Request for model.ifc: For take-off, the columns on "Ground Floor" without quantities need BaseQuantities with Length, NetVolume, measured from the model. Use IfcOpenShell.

First a look at what the model holds.

```python
import ifcopenshell
import ifcopenshell.util.element
import ifcopenshell.util.unit

model = ifcopenshell.open("model.ifc")
print(model.schema)
for unit_type in ("LENGTHUNIT", "AREAUNIT", "VOLUMEUNIT"):
    print(unit_type, ifcopenshell.util.unit.calculate_unit_scale(model, unit_type))
storey = next(s for s in model.by_type("IfcBuildingStorey") if s.Name == "Ground Floor")
columns = [e for e in ifcopenshell.util.element.get_decomposition(storey) if e.is_a("IfcColumn")]
for e in sorted(columns, key=lambda e: e.id()):
    print(e.id(), e.is_a(), e.Name, list(ifcopenshell.util.element.get_psets(e, qtos_only=True)), sep=" | ")
```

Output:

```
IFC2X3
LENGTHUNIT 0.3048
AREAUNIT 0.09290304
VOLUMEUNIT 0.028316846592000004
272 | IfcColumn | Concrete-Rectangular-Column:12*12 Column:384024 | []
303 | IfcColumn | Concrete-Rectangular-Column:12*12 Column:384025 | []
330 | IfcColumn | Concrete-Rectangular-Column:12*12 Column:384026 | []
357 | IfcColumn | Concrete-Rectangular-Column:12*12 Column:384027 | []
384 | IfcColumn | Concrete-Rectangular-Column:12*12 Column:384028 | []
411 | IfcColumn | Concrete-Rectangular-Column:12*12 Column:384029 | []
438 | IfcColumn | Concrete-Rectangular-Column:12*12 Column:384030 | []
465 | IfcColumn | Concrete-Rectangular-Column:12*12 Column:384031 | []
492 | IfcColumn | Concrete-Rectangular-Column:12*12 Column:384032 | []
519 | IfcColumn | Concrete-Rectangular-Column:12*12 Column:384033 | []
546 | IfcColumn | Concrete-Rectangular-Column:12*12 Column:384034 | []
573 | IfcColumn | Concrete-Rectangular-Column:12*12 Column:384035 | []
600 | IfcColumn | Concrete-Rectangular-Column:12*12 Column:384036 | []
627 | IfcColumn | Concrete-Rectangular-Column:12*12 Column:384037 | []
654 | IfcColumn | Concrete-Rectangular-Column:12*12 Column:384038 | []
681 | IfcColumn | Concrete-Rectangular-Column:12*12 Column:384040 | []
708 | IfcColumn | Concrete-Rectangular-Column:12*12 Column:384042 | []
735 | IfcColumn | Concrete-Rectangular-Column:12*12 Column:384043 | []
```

```python
import ifcopenshell
import ifcopenshell.api.pset
import ifcopenshell.geom
import ifcopenshell.util.element
import ifcopenshell.util.shape
import ifcopenshell.util.unit

model = ifcopenshell.open("model.ifc")
unit_scale = ifcopenshell.util.unit.calculate_unit_scale(model)
volume_scale = ifcopenshell.util.unit.calculate_unit_scale(model, "VOLUMEUNIT")
settings = ifcopenshell.geom.settings()

storey = next(s for s in model.by_type("IfcBuildingStorey") if s.Name == "Ground Floor")
columns = [e for e in ifcopenshell.util.element.get_decomposition(storey) if e.is_a("IfcColumn")]

for e in sorted(columns, key=lambda e: e.id()):
    if ifcopenshell.util.element.get_psets(e, qtos_only=True, should_inherit=False):
        continue
    # Geometry comes back in metres, in the element's own axes.
    shape = ifcopenshell.geom.create_shape(settings, e)
    values = {
        "Length": ifcopenshell.util.shape.get_z(shape.geometry) / unit_scale,
        "NetVolume": ifcopenshell.util.shape.get_volume(shape.geometry) / volume_scale,
    }
    qto = ifcopenshell.api.pset.add_qto(model, product=e, name="BaseQuantities")
    ifcopenshell.api.pset.edit_qto(model, qto=qto, properties=values)
    print(e.id(), {k: round(v, 3) for k, v in values.items()})

model.write("model_rev.ifc")
```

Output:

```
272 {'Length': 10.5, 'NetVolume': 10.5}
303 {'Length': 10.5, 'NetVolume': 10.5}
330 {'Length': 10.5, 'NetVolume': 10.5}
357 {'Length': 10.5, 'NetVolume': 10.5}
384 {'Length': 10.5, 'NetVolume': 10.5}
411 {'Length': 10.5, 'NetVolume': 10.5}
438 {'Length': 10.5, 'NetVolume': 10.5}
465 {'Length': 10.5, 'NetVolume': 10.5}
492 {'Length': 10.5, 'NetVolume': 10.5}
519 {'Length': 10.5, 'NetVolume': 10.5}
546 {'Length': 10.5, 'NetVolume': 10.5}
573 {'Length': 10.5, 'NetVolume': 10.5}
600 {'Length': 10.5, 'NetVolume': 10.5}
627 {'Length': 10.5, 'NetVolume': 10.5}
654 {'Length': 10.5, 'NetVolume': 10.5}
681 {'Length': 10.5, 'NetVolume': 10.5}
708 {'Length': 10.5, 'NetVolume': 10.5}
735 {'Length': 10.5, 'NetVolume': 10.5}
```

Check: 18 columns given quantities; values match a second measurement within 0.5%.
